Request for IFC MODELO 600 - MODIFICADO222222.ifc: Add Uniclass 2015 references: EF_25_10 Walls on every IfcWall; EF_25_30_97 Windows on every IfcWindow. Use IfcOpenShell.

First a look at what the model holds.

```python
import ifcopenshell

model = ifcopenshell.open("IFC MODELO 600 - MODIFICADO222222.ifc")
print(model.schema)
print("classifications:", [c.Name for c in model.by_type("IfcClassification")])
for ifc_class in ("IfcDoor", "IfcRoof", "IfcStair", "IfcWall", "IfcWindow"):
    print(ifc_class, len(model.by_type(ifc_class)))
```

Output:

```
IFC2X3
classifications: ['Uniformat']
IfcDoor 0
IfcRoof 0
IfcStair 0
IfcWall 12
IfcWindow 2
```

```python
import ifcopenshell
import ifcopenshell.api.classification

model = ifcopenshell.open("IFC MODELO 600 - MODIFICADO222222.ifc")

# IFC2X3 requires Source and Edition and has no link from the project to the system.
system = model.create_entity("IfcClassification", Source="NBS", Edition="2015", Name="Uniclass 2015")

codes = {
    "IfcWall": ("EF_25_10", "Walls"),
    "IfcWindow": ("EF_25_30_97", "Windows"),
}
for ifc_class, (code, name) in codes.items():
    products = model.by_type(ifc_class)
    ifcopenshell.api.classification.add_reference(
        model, products=products, classification=system, identification=code, name=name
    )
    print(code, len(products))

model.write("IFC MODELO 600 - MODIFICADO222222_rev.ifc")
```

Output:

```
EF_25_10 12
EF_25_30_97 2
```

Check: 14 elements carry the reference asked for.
